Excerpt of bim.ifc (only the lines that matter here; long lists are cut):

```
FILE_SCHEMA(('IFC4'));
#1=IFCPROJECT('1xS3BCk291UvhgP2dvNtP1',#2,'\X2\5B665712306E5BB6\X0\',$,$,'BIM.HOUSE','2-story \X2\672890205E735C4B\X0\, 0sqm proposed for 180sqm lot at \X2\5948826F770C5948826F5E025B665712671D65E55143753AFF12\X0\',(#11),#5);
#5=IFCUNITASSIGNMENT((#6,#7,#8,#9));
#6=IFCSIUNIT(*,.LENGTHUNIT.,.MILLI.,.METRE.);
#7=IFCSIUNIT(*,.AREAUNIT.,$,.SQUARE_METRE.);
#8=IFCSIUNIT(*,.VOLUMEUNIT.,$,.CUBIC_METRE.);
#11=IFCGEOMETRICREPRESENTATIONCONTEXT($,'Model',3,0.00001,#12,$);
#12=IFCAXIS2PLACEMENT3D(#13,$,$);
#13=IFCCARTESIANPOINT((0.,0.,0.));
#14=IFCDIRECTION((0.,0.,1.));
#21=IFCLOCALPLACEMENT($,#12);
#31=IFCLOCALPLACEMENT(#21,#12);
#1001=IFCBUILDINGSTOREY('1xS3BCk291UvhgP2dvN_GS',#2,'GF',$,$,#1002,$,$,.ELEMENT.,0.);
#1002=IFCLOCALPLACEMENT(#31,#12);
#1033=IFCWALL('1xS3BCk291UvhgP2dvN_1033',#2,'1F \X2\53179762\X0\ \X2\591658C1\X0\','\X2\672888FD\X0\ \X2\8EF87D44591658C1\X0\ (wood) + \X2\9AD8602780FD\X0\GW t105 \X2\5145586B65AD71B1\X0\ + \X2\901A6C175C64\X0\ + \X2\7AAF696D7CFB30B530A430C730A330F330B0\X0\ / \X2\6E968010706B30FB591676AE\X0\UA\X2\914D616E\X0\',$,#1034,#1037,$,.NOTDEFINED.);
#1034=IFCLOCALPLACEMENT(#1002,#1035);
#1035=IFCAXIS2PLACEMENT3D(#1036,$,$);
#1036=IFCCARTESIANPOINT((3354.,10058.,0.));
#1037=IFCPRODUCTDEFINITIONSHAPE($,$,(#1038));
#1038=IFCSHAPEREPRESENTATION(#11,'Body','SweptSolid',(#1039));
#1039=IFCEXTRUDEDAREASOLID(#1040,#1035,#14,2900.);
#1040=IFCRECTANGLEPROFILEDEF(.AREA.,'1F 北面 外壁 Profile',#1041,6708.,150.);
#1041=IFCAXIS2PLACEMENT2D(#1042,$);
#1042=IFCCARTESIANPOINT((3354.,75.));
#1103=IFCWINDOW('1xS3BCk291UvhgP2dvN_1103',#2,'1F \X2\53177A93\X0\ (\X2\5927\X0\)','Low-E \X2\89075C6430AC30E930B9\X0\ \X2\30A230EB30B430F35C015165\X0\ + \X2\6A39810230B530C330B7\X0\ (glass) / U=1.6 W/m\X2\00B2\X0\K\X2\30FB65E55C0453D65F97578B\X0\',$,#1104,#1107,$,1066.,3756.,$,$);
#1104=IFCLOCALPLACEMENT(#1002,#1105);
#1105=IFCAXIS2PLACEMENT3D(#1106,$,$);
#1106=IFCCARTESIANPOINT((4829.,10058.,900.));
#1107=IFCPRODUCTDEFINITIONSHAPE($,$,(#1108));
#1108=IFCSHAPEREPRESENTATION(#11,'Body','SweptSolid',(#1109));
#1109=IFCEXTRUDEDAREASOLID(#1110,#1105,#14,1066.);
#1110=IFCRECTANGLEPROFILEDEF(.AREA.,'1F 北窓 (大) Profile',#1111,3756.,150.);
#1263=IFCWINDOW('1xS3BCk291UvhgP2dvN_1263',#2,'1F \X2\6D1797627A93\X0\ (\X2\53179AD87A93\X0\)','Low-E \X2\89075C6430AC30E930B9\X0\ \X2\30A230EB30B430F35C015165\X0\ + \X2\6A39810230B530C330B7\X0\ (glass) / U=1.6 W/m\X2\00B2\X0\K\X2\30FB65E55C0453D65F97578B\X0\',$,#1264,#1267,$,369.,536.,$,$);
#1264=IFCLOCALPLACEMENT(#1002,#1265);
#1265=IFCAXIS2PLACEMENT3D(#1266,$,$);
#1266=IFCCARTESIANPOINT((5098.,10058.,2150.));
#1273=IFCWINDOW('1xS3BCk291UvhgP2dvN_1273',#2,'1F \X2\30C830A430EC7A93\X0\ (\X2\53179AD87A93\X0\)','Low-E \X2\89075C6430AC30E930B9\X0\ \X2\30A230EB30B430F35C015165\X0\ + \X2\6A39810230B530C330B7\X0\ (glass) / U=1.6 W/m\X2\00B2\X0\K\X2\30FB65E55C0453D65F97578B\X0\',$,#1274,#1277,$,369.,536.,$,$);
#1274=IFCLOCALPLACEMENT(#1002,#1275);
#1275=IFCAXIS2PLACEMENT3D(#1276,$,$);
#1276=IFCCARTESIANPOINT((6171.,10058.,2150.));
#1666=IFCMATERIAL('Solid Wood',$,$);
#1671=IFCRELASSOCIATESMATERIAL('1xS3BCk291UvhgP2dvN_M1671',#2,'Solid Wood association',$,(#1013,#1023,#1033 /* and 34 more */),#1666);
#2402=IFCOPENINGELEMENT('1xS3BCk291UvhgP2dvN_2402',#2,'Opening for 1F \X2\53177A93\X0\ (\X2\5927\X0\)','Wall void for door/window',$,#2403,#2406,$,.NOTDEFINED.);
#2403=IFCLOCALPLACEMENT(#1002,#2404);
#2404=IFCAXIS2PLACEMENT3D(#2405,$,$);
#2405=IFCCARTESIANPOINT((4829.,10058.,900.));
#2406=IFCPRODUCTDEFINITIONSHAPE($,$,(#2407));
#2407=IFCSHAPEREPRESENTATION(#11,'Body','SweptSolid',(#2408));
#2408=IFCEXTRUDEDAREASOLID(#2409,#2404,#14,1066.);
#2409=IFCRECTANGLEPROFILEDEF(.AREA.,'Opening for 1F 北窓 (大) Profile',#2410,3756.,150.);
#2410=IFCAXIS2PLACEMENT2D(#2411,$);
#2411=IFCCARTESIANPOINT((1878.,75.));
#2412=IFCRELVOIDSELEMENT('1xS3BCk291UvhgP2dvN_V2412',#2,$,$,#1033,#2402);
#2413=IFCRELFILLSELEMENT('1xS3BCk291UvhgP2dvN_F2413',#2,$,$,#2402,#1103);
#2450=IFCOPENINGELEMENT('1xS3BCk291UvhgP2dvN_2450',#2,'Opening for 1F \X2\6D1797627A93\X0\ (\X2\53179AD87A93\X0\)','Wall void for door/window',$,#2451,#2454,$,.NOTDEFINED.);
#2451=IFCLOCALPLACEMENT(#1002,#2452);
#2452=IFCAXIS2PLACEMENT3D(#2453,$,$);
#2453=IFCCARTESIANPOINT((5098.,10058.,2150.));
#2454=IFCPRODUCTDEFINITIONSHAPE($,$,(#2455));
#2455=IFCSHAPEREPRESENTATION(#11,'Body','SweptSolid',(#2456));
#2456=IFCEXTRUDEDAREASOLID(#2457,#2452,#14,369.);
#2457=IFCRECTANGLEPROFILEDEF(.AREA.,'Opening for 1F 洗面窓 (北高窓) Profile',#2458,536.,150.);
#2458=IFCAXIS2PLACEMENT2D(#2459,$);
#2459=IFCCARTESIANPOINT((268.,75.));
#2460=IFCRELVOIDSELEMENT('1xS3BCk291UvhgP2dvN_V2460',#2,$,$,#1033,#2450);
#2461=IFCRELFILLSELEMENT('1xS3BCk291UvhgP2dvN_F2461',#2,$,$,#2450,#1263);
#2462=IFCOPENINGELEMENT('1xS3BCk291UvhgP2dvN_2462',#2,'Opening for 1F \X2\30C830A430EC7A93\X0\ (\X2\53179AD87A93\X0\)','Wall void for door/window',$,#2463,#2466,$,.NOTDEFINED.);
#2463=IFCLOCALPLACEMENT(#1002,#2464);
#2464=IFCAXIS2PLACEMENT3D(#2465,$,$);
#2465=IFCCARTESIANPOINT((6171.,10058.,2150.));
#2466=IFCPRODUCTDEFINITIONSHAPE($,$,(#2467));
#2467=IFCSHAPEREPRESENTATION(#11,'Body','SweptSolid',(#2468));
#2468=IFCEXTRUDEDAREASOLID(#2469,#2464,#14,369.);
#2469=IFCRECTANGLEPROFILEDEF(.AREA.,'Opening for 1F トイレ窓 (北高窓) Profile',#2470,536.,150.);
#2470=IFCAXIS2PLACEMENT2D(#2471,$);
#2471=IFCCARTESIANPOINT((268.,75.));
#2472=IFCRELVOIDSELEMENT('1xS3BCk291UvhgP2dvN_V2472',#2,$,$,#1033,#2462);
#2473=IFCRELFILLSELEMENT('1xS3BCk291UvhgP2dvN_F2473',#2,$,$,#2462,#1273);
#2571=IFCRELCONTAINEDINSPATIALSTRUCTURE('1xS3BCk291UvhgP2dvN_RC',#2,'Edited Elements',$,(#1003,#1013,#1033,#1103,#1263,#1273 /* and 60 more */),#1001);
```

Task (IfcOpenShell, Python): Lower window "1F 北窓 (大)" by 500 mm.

```python
import numpy as np
import ifcopenshell
import ifcopenshell.api.geometry
import ifcopenshell.util.placement
import ifcopenshell.util.unit

model = ifcopenshell.open("bim.ifc")
unit_scale = ifcopenshell.util.unit.calculate_unit_scale(model)

window = model.by_guid("1xS3BCk291UvhgP2dvN_1103")
opening = window.FillsVoids[0].RelatingOpeningElement
dz = -500.0

shift = np.array([0.0, 0.0, dz])
# The window is not placed relative to its opening, so move both.
for product in (opening, window):
    matrix = ifcopenshell.util.placement.get_local_placement(product.ObjectPlacement)
    matrix[:3, 3] += shift
    ifcopenshell.api.geometry.edit_object_placement(model, product=product, matrix=matrix, is_si=False)

print(f"moved by {dz * unit_scale:+.3f} m")

model.write("bim_edited.ifc")
```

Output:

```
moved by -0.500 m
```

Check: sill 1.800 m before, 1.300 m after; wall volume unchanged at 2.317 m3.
